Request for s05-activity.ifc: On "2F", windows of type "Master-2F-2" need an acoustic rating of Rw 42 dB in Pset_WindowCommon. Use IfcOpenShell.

First a look at what the model holds.

```python
import ifcopenshell
import ifcopenshell.util.element

model = ifcopenshell.open("s05-activity.ifc")
print(model.schema)
storey = next(s for s in model.by_type("IfcBuildingStorey") if s.Name == "2F")
windows = [e for e in ifcopenshell.util.element.get_decomposition(storey) if e.is_a("IfcWindow")]
seen = {}
for e in windows:
    element_type = ifcopenshell.util.element.get_type(e)
    key = (element_type.Name if element_type != e and element_type else None, ifcopenshell.util.element.get_pset(e, "Pset_WindowCommon", "AcousticRating"))
    seen[key] = seen.get(key, 0) + 1
for (name, value), count in sorted(seen.items(), key=str):
    print(count, "x", name, "|", value)
```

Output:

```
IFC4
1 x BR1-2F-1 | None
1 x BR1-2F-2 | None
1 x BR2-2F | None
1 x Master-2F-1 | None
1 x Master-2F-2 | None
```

```python
import ifcopenshell
import ifcopenshell.api.pset
import ifcopenshell.util.element

model = ifcopenshell.open("s05-activity.ifc")

storey = next(s for s in model.by_type("IfcBuildingStorey") if s.Name == "2F")
windows = [e for e in ifcopenshell.util.element.get_decomposition(storey) if e.is_a("IfcWindow")]

count = 0
for e in windows:
    element_type = ifcopenshell.util.element.get_type(e)
    if element_type in (None, e) or element_type.Name != "Master-2F-2":
        continue
    # add_pset returns the element's existing set when there is one.
    pset = ifcopenshell.api.pset.add_pset(model, product=e, name="Pset_WindowCommon")
    ifcopenshell.api.pset.edit_pset(model, pset=pset, properties={"AcousticRating": "Rw 42 dB"})
    count += 1

print(count, "windows updated")

model.write("s05-activity-out.ifc")
```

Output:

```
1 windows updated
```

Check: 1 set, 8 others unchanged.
